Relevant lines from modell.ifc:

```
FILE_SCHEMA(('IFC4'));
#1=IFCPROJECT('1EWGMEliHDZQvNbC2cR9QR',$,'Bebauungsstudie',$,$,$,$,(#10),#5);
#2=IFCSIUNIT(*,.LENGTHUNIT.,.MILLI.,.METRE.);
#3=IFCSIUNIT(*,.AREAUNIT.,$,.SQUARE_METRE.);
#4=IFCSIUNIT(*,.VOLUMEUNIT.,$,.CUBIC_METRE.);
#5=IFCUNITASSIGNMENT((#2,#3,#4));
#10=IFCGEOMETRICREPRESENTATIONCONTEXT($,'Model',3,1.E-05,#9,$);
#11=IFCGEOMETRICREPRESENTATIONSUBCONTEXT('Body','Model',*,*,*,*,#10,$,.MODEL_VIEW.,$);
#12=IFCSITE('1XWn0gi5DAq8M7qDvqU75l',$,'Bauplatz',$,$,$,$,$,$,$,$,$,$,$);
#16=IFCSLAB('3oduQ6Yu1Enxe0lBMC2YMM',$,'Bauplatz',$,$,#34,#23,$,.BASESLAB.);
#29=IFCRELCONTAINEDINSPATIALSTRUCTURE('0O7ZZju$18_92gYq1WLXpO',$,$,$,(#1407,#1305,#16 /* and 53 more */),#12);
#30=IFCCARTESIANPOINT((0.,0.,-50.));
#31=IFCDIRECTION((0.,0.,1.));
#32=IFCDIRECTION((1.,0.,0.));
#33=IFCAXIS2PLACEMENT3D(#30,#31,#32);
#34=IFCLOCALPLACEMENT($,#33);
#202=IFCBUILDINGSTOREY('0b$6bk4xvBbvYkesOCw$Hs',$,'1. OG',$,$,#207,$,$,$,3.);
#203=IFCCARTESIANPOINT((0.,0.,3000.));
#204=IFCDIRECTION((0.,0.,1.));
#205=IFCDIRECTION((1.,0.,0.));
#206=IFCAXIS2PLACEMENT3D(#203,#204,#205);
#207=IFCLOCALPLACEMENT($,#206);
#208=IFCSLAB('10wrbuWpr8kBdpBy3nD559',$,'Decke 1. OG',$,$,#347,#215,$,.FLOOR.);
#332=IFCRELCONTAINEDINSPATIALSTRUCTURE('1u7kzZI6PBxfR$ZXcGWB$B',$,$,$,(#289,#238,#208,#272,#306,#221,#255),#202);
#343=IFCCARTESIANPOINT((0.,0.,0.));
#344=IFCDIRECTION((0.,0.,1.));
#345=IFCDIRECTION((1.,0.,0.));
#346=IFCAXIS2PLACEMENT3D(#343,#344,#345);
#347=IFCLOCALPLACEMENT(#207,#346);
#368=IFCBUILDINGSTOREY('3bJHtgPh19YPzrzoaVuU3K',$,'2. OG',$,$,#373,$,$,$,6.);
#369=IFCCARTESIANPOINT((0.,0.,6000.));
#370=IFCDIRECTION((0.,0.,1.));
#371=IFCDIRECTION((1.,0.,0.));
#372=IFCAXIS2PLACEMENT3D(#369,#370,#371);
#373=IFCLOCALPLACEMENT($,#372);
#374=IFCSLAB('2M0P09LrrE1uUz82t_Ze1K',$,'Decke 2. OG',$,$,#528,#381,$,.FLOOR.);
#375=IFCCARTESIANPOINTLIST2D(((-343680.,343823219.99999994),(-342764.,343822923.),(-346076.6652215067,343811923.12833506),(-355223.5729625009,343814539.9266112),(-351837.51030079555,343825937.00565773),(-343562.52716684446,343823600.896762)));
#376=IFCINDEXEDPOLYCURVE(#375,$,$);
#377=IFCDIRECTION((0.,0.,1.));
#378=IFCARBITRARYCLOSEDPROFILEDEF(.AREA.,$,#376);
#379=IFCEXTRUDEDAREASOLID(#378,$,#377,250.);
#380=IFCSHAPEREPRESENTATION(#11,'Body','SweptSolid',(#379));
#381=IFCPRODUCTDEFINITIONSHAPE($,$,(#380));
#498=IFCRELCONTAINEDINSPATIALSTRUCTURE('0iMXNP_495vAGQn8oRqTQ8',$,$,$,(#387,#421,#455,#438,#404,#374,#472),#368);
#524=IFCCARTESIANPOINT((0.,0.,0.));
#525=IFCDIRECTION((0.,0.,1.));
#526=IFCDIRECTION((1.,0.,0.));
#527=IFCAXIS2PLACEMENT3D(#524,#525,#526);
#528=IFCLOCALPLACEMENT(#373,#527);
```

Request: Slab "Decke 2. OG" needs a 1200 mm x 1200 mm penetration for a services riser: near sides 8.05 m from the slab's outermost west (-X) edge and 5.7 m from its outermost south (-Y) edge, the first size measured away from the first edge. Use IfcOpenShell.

```python
import numpy as np
import ifcopenshell
import ifcopenshell.api.feature
import ifcopenshell.api.geometry
import ifcopenshell.api.root
import ifcopenshell.geom
import ifcopenshell.util.placement
import ifcopenshell.util.representation
import ifcopenshell.util.shape
import ifcopenshell.util.unit

model = ifcopenshell.open("modell.ifc")
unit_scale = ifcopenshell.util.unit.calculate_unit_scale(model)
settings = ifcopenshell.geom.settings()


def volume(element):
    """Net volume in cubic metres, openings subtracted."""
    shape = ifcopenshell.geom.create_shape(settings, element)
    return ifcopenshell.util.shape.get_volume(shape.geometry)


slab = model.by_guid("2M0P09LrrE1uUz82t_Ze1K")
before = volume(slab)

# Extent in the slab's own axes, in metres. The edges named are its -X and -Y sides.
slab_shape = ifcopenshell.geom.create_shape(settings, slab)
vertices = ifcopenshell.util.shape.get_vertices(slab_shape.geometry)
x_min, y_min, bottom = vertices.min(axis=0)
top = vertices[:, 2].max()

opening = ifcopenshell.api.root.create_entity(model, ifc_class="IfcOpeningElement", name="Services riser opening", predefined_type="OPENING")
context = ifcopenshell.util.representation.get_context(model, "Model", "Body", "MODEL_VIEW")
width, depth = 1.2, 1.2
outline = [(0.0, 0.0), (width, 0.0), (width, depth), (0.0, depth), (0.0, 0.0)]
# Overshoot both faces by 50 mm so the cut is clean.
shape = ifcopenshell.api.geometry.add_slab_representation(
    model, context=context, depth=top - bottom + 0.1, polyline=outline
)
ifcopenshell.api.geometry.assign_representation(model, product=opening, representation=shape)

matrix = ifcopenshell.util.placement.get_local_placement(slab.ObjectPlacement)
matrix[:, 3] = matrix @ np.append(np.array([x_min + 8.05, y_min + 5.7, bottom - 0.05]) / unit_scale, 1.0)
ifcopenshell.api.geometry.edit_object_placement(model, product=opening, matrix=matrix, is_si=False)
ifcopenshell.api.feature.add_feature(model, feature=opening, element=slab)

after = volume(slab)

print(f"slab volume {before:.3f} -> {after:.3f} m3")

model.write("modell_v2.ifc")
```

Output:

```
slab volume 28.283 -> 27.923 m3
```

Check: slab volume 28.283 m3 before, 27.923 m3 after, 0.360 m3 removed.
